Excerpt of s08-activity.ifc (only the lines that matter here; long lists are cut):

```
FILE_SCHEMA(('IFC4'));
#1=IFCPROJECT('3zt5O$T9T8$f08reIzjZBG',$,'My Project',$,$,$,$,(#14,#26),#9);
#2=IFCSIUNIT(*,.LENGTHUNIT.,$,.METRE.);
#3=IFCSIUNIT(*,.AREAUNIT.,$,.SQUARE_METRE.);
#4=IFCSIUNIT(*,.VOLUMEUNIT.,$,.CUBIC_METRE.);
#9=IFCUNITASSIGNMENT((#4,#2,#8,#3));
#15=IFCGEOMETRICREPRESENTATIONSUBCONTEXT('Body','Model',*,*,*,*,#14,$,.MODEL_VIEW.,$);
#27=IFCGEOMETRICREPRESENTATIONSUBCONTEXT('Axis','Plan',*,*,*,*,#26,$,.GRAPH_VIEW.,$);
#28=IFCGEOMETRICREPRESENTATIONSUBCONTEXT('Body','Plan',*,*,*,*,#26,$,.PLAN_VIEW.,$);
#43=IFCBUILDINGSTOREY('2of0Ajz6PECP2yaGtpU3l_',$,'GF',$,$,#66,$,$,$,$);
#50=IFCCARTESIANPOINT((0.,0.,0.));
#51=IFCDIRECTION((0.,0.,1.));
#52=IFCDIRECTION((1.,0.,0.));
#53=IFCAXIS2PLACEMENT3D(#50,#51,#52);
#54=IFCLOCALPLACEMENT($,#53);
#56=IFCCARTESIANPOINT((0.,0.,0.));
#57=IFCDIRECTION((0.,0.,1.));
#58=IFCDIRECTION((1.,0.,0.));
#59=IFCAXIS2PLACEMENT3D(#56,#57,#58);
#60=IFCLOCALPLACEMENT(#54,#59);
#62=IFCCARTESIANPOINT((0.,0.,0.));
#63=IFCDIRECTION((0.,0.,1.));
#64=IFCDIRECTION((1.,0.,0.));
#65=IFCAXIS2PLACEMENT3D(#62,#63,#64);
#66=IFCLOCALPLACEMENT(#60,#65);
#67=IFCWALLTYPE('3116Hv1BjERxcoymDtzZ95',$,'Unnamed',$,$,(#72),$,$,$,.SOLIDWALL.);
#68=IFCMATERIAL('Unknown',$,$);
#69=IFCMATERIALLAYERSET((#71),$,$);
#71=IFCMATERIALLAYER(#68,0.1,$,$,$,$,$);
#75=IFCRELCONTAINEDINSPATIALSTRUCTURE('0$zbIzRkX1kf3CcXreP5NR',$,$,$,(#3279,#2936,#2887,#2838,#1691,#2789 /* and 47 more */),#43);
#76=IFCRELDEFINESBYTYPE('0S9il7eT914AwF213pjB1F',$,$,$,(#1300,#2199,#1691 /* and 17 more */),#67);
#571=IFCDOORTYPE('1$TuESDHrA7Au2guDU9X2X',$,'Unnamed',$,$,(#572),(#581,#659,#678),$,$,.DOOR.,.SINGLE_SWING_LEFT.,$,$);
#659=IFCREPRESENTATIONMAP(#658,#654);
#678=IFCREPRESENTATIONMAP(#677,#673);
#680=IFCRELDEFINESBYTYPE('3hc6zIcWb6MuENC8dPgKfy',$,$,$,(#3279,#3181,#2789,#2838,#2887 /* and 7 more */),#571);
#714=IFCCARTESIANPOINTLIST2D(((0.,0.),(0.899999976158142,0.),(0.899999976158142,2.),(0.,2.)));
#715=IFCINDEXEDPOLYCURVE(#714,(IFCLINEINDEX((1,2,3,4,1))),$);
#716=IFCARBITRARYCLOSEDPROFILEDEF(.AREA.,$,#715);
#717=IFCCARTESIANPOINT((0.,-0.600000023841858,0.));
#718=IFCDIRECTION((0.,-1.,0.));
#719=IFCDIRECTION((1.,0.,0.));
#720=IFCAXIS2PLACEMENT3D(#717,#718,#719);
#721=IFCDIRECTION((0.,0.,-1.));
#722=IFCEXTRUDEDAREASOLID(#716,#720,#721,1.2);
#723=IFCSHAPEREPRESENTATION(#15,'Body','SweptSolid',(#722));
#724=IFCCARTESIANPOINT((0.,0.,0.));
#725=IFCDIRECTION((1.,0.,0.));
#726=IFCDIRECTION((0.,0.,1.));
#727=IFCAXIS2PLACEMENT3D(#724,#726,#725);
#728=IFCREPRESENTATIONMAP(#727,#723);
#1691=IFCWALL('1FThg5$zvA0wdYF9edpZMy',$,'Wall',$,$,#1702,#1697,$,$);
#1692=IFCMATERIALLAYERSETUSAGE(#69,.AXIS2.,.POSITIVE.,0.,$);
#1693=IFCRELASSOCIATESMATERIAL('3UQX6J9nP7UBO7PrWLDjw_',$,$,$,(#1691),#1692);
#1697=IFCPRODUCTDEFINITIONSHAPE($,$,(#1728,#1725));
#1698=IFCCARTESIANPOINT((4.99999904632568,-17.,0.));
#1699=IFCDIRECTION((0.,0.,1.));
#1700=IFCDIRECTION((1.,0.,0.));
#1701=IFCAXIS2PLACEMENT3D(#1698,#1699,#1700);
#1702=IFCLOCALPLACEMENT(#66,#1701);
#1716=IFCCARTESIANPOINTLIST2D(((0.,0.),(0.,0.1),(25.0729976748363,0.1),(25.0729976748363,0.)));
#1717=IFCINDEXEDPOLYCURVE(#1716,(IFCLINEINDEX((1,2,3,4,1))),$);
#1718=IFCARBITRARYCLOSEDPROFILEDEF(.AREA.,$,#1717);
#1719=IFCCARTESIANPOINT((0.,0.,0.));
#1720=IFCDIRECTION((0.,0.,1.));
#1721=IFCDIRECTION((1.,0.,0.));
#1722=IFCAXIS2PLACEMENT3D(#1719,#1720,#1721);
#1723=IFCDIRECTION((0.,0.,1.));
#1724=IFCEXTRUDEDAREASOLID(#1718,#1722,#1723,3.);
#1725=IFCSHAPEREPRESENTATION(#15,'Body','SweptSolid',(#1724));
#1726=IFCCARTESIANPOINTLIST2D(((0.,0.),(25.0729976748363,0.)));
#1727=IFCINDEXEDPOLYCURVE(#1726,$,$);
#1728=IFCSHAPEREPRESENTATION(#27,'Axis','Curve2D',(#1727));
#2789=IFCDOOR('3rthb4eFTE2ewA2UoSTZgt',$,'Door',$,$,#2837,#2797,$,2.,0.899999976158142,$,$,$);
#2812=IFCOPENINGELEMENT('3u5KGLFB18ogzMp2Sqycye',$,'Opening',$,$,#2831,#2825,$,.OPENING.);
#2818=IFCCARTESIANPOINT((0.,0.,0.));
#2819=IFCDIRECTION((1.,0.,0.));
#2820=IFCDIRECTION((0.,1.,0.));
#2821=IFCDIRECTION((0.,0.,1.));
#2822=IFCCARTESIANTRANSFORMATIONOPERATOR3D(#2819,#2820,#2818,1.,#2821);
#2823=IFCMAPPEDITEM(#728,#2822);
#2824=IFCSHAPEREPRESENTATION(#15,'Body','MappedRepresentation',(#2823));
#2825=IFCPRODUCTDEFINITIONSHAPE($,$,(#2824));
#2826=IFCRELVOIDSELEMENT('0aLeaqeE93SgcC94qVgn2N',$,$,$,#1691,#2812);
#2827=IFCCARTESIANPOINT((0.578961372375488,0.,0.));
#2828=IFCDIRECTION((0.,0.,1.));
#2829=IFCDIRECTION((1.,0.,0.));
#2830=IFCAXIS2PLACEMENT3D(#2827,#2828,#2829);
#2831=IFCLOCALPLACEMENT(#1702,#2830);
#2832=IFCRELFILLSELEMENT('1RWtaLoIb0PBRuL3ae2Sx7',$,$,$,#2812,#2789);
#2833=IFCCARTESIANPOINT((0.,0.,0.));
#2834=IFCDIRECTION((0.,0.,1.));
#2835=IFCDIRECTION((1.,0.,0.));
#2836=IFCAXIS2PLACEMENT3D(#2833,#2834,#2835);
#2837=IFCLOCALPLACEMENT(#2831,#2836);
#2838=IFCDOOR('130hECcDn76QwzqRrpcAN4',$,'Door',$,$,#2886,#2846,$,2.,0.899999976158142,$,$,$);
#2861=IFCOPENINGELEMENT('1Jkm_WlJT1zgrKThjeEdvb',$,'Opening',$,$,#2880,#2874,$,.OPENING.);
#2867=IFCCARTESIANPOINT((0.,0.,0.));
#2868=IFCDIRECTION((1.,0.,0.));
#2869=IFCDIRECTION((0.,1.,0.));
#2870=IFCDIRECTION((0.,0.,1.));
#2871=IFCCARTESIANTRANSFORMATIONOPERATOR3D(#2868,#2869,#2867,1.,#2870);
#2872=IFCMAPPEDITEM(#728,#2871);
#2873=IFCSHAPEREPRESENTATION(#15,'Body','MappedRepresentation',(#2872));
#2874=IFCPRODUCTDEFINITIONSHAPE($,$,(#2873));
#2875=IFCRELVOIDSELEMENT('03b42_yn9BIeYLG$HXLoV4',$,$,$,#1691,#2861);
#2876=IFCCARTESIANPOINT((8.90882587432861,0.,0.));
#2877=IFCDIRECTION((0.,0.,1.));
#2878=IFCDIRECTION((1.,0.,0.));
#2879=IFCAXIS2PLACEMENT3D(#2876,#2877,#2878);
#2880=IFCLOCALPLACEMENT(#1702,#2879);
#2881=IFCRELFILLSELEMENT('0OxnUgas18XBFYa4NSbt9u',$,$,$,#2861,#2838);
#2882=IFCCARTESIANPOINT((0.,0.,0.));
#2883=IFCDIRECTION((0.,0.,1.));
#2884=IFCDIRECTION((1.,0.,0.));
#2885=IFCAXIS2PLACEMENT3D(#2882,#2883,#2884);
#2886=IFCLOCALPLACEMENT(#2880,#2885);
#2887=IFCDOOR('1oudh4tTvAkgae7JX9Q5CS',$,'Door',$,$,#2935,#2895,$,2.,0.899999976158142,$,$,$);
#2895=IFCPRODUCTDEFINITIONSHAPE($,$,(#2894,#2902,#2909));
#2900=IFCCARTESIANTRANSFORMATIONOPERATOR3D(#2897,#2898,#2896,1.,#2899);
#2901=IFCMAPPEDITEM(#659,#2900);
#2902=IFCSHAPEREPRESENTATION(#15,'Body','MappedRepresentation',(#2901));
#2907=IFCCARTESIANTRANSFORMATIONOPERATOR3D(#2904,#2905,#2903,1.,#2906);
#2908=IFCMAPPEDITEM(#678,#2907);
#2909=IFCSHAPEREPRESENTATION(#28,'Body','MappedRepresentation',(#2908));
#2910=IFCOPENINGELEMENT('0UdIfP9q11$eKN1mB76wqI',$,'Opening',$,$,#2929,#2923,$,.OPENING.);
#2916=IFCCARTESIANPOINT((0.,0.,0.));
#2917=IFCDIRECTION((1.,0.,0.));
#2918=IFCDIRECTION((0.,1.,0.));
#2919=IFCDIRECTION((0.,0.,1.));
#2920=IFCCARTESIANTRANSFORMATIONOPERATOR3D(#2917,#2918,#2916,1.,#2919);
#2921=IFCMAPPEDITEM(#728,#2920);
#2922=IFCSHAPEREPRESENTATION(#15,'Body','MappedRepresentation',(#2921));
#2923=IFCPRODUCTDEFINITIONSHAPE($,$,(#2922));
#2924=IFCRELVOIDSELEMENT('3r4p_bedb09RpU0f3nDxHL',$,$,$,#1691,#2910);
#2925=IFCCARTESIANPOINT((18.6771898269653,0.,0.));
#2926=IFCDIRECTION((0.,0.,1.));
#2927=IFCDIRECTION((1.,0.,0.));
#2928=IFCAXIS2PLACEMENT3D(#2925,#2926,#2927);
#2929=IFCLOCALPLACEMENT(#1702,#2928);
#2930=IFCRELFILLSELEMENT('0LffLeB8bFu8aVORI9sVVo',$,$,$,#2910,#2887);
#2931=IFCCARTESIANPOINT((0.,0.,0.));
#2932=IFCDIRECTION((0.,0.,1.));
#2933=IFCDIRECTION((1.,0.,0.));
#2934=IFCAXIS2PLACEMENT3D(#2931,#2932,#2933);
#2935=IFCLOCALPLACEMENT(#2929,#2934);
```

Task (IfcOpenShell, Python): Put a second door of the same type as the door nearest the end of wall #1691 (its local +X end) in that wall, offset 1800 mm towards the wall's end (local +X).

```python
import ifcopenshell
import ifcopenshell.api.feature
import ifcopenshell.api.geometry
import ifcopenshell.api.root
import ifcopenshell.geom
import ifcopenshell.util.element
import ifcopenshell.util.placement
import ifcopenshell.util.shape

model = ifcopenshell.open("s08-activity.ifc")
settings = ifcopenshell.geom.settings()


def volume(element):
    """Net volume in cubic metres, openings subtracted."""
    shape = ifcopenshell.geom.create_shape(settings, element)
    return ifcopenshell.util.shape.get_volume(shape.geometry)


door = model.by_guid("1oudh4tTvAkgae7JX9Q5CS")
opening = door.FillsVoids[0].RelatingOpeningElement
wall = opening.VoidsElements[0].RelatingBuildingElement
before = volume(wall)
shift = ifcopenshell.util.placement.get_local_placement(wall.ObjectPlacement)[:3, 0] * 1.8

# copy_class copies the void relationship, type, container and properties, but no geometry.
new_opening = ifcopenshell.api.root.copy_class(model, product=opening)
new_opening.Representation = ifcopenshell.util.element.copy_deep(
    model, opening.Representation, exclude=["IfcGeometricRepresentationContext", "IfcRepresentationMap"]
)
new_door = ifcopenshell.api.root.copy_class(model, product=door)
new_door.Representation = ifcopenshell.util.element.copy_deep(
    model, door.Representation, exclude=["IfcGeometricRepresentationContext", "IfcRepresentationMap"]
)
ifcopenshell.api.feature.add_filling(model, opening=new_opening, element=new_door)

for old, new in ((opening, new_opening), (door, new_door)):
    matrix = ifcopenshell.util.placement.get_local_placement(old.ObjectPlacement)
    matrix[:3, 3] += shift
    ifcopenshell.api.geometry.edit_object_placement(model, product=new, matrix=matrix, is_si=False)

after = volume(wall)

print(f"wall volume {before:.3f} -> {after:.3f} m3")

model.write("s08-activity-out.ifc")
```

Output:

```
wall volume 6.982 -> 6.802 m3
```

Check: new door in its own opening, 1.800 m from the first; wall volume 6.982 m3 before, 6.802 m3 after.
